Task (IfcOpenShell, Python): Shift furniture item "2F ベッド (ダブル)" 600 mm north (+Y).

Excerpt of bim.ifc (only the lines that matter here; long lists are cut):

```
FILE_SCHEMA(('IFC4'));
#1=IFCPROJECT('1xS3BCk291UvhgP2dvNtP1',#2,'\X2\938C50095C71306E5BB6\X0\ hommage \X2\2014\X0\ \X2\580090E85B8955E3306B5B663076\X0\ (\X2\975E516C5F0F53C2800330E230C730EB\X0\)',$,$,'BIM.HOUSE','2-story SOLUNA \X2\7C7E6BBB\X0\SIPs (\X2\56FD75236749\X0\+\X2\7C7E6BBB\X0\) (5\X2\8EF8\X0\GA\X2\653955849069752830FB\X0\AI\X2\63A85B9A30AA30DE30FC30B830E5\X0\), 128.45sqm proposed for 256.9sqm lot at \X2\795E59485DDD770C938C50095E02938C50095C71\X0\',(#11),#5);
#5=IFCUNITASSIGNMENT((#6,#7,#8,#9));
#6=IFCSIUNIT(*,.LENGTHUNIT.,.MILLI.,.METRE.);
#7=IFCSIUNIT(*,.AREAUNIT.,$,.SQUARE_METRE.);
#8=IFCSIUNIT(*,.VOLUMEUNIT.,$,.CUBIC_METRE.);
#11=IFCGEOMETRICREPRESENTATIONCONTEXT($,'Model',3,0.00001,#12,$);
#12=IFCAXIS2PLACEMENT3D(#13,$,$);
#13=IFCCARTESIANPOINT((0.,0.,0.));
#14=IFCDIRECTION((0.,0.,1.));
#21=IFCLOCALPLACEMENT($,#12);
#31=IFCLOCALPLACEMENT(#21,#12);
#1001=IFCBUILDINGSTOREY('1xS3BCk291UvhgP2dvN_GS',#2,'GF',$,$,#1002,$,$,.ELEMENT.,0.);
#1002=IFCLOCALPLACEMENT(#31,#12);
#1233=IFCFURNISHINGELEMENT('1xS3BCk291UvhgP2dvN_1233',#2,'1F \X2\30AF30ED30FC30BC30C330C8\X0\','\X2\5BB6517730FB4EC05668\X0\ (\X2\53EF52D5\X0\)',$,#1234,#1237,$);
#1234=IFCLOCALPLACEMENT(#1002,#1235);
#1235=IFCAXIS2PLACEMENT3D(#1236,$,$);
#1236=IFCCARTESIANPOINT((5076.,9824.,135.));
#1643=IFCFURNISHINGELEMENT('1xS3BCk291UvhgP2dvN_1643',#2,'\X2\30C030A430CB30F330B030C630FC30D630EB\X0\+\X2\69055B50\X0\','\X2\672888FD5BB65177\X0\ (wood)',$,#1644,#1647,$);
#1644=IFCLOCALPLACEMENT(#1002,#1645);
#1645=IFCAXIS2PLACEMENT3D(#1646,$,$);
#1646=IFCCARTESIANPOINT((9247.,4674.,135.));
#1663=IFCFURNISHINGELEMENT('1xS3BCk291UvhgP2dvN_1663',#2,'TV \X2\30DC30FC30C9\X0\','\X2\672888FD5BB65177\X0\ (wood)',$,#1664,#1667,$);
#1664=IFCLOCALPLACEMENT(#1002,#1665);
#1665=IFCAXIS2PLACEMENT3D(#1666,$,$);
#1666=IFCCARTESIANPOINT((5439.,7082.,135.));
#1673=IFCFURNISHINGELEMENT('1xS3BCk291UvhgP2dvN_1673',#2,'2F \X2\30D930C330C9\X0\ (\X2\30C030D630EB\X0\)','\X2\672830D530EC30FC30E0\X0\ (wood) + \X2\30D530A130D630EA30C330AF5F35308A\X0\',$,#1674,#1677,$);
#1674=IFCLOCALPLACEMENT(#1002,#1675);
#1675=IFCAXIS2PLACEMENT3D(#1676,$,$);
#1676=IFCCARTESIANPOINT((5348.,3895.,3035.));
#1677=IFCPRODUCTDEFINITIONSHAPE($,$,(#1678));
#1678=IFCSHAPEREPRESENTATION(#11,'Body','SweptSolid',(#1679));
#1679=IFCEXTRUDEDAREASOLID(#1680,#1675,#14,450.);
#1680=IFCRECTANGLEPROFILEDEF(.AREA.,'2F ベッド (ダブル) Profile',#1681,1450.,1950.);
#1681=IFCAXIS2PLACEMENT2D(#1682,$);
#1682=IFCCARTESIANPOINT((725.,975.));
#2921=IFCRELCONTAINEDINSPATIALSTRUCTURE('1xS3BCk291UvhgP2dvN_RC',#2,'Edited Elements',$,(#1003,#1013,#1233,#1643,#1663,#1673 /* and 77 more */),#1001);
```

```python
import ifcopenshell
import ifcopenshell.api.geometry
import ifcopenshell.util.placement
import ifcopenshell.util.unit

model = ifcopenshell.open("bim.ifc")
unit_scale = ifcopenshell.util.unit.calculate_unit_scale(model)

item = model.by_id(1673)
matrix = ifcopenshell.util.placement.get_local_placement(item.ObjectPlacement)
matrix[1, 3] += 0.6 / unit_scale
ifcopenshell.api.geometry.edit_object_placement(model, product=item, matrix=matrix, is_si=False)

print(ifcopenshell.util.placement.get_local_placement(item.ObjectPlacement).round(3) + 0.0)

model.write("bim_v2.ifc")
```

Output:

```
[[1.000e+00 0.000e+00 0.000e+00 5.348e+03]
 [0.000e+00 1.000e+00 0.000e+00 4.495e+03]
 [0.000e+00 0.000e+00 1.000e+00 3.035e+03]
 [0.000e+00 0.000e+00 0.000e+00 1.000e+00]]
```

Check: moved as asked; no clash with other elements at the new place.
